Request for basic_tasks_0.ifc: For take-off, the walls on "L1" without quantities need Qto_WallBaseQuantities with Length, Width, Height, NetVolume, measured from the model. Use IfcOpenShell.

First a look at what the model holds.

```python
import ifcopenshell
import ifcopenshell.util.element
import ifcopenshell.util.unit

model = ifcopenshell.open("basic_tasks_0.ifc")
print(model.schema)
for unit_type in ("LENGTHUNIT", "AREAUNIT", "VOLUMEUNIT"):
    print(unit_type, ifcopenshell.util.unit.calculate_unit_scale(model, unit_type))
storey = next(s for s in model.by_type("IfcBuildingStorey") if s.Name == "L1")
walls = [e for e in ifcopenshell.util.element.get_decomposition(storey) if e.is_a("IfcWall")]
for e in sorted(walls, key=lambda e: e.id()):
    print(e.id(), e.is_a(), e.Name, list(ifcopenshell.util.element.get_psets(e, qtos_only=True)), sep=" | ")
```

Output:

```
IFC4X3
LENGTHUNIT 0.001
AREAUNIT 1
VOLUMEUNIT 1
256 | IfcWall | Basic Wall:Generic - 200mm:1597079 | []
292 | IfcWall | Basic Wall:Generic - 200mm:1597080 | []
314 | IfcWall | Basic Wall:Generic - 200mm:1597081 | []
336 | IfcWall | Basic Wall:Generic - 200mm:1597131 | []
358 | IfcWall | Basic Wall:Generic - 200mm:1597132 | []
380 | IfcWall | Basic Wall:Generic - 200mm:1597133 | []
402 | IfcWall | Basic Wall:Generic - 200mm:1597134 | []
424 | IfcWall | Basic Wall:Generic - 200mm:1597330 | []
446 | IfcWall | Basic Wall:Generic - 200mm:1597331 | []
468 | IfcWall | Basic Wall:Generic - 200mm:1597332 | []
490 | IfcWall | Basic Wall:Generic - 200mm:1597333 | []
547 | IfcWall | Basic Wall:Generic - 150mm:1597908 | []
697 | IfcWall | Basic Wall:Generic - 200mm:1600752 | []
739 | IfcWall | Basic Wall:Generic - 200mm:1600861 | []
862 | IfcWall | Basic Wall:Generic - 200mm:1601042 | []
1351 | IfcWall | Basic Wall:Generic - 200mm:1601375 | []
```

```python
import ifcopenshell
import ifcopenshell.api.pset
import ifcopenshell.geom
import ifcopenshell.util.element
import ifcopenshell.util.shape
import ifcopenshell.util.unit

model = ifcopenshell.open("basic_tasks_0.ifc")
unit_scale = ifcopenshell.util.unit.calculate_unit_scale(model)
volume_scale = ifcopenshell.util.unit.calculate_unit_scale(model, "VOLUMEUNIT")
settings = ifcopenshell.geom.settings()

storey = next(s for s in model.by_type("IfcBuildingStorey") if s.Name == "L1")
walls = [e for e in ifcopenshell.util.element.get_decomposition(storey) if e.is_a("IfcWall")]

for e in sorted(walls, key=lambda e: e.id()):
    if ifcopenshell.util.element.get_psets(e, qtos_only=True, should_inherit=False):
        continue
    # Geometry comes back in metres, in the element's own axes.
    shape = ifcopenshell.geom.create_shape(settings, e)
    values = {
        "Length": ifcopenshell.util.shape.get_x(shape.geometry) / unit_scale,
        "Width": ifcopenshell.util.shape.get_y(shape.geometry) / unit_scale,
        "Height": ifcopenshell.util.shape.get_z(shape.geometry) / unit_scale,
        "NetVolume": ifcopenshell.util.shape.get_volume(shape.geometry) / volume_scale,
    }
    qto = ifcopenshell.api.pset.add_qto(model, product=e, name="Qto_WallBaseQuantities")
    ifcopenshell.api.pset.edit_qto(model, qto=qto, properties=values)
    print(e.id(), {k: round(v, 3) for k, v in values.items()})

model.write("basic_tasks_0_rev.ifc")
```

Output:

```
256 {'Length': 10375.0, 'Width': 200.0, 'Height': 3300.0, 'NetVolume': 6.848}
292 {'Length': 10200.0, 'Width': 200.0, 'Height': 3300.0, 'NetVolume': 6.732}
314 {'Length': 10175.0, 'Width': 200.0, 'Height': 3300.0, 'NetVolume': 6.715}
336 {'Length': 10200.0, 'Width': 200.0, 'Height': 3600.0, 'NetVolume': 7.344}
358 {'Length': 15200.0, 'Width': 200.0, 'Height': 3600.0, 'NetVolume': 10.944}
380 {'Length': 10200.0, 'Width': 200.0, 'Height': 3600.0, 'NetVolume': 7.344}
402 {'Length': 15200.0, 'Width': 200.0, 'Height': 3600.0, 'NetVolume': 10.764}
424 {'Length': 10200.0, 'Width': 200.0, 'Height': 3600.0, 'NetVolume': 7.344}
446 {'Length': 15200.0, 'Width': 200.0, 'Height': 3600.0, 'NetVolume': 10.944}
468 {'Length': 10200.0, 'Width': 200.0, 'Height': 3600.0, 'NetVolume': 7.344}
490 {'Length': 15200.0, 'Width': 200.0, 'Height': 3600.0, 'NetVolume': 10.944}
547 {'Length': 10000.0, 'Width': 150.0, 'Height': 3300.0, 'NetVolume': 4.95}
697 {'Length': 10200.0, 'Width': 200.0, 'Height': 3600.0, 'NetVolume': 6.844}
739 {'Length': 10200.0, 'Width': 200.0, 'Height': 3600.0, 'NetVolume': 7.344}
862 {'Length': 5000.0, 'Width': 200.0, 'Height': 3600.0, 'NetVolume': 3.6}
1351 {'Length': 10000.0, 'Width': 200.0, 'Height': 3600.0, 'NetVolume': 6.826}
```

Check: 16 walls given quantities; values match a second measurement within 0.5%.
